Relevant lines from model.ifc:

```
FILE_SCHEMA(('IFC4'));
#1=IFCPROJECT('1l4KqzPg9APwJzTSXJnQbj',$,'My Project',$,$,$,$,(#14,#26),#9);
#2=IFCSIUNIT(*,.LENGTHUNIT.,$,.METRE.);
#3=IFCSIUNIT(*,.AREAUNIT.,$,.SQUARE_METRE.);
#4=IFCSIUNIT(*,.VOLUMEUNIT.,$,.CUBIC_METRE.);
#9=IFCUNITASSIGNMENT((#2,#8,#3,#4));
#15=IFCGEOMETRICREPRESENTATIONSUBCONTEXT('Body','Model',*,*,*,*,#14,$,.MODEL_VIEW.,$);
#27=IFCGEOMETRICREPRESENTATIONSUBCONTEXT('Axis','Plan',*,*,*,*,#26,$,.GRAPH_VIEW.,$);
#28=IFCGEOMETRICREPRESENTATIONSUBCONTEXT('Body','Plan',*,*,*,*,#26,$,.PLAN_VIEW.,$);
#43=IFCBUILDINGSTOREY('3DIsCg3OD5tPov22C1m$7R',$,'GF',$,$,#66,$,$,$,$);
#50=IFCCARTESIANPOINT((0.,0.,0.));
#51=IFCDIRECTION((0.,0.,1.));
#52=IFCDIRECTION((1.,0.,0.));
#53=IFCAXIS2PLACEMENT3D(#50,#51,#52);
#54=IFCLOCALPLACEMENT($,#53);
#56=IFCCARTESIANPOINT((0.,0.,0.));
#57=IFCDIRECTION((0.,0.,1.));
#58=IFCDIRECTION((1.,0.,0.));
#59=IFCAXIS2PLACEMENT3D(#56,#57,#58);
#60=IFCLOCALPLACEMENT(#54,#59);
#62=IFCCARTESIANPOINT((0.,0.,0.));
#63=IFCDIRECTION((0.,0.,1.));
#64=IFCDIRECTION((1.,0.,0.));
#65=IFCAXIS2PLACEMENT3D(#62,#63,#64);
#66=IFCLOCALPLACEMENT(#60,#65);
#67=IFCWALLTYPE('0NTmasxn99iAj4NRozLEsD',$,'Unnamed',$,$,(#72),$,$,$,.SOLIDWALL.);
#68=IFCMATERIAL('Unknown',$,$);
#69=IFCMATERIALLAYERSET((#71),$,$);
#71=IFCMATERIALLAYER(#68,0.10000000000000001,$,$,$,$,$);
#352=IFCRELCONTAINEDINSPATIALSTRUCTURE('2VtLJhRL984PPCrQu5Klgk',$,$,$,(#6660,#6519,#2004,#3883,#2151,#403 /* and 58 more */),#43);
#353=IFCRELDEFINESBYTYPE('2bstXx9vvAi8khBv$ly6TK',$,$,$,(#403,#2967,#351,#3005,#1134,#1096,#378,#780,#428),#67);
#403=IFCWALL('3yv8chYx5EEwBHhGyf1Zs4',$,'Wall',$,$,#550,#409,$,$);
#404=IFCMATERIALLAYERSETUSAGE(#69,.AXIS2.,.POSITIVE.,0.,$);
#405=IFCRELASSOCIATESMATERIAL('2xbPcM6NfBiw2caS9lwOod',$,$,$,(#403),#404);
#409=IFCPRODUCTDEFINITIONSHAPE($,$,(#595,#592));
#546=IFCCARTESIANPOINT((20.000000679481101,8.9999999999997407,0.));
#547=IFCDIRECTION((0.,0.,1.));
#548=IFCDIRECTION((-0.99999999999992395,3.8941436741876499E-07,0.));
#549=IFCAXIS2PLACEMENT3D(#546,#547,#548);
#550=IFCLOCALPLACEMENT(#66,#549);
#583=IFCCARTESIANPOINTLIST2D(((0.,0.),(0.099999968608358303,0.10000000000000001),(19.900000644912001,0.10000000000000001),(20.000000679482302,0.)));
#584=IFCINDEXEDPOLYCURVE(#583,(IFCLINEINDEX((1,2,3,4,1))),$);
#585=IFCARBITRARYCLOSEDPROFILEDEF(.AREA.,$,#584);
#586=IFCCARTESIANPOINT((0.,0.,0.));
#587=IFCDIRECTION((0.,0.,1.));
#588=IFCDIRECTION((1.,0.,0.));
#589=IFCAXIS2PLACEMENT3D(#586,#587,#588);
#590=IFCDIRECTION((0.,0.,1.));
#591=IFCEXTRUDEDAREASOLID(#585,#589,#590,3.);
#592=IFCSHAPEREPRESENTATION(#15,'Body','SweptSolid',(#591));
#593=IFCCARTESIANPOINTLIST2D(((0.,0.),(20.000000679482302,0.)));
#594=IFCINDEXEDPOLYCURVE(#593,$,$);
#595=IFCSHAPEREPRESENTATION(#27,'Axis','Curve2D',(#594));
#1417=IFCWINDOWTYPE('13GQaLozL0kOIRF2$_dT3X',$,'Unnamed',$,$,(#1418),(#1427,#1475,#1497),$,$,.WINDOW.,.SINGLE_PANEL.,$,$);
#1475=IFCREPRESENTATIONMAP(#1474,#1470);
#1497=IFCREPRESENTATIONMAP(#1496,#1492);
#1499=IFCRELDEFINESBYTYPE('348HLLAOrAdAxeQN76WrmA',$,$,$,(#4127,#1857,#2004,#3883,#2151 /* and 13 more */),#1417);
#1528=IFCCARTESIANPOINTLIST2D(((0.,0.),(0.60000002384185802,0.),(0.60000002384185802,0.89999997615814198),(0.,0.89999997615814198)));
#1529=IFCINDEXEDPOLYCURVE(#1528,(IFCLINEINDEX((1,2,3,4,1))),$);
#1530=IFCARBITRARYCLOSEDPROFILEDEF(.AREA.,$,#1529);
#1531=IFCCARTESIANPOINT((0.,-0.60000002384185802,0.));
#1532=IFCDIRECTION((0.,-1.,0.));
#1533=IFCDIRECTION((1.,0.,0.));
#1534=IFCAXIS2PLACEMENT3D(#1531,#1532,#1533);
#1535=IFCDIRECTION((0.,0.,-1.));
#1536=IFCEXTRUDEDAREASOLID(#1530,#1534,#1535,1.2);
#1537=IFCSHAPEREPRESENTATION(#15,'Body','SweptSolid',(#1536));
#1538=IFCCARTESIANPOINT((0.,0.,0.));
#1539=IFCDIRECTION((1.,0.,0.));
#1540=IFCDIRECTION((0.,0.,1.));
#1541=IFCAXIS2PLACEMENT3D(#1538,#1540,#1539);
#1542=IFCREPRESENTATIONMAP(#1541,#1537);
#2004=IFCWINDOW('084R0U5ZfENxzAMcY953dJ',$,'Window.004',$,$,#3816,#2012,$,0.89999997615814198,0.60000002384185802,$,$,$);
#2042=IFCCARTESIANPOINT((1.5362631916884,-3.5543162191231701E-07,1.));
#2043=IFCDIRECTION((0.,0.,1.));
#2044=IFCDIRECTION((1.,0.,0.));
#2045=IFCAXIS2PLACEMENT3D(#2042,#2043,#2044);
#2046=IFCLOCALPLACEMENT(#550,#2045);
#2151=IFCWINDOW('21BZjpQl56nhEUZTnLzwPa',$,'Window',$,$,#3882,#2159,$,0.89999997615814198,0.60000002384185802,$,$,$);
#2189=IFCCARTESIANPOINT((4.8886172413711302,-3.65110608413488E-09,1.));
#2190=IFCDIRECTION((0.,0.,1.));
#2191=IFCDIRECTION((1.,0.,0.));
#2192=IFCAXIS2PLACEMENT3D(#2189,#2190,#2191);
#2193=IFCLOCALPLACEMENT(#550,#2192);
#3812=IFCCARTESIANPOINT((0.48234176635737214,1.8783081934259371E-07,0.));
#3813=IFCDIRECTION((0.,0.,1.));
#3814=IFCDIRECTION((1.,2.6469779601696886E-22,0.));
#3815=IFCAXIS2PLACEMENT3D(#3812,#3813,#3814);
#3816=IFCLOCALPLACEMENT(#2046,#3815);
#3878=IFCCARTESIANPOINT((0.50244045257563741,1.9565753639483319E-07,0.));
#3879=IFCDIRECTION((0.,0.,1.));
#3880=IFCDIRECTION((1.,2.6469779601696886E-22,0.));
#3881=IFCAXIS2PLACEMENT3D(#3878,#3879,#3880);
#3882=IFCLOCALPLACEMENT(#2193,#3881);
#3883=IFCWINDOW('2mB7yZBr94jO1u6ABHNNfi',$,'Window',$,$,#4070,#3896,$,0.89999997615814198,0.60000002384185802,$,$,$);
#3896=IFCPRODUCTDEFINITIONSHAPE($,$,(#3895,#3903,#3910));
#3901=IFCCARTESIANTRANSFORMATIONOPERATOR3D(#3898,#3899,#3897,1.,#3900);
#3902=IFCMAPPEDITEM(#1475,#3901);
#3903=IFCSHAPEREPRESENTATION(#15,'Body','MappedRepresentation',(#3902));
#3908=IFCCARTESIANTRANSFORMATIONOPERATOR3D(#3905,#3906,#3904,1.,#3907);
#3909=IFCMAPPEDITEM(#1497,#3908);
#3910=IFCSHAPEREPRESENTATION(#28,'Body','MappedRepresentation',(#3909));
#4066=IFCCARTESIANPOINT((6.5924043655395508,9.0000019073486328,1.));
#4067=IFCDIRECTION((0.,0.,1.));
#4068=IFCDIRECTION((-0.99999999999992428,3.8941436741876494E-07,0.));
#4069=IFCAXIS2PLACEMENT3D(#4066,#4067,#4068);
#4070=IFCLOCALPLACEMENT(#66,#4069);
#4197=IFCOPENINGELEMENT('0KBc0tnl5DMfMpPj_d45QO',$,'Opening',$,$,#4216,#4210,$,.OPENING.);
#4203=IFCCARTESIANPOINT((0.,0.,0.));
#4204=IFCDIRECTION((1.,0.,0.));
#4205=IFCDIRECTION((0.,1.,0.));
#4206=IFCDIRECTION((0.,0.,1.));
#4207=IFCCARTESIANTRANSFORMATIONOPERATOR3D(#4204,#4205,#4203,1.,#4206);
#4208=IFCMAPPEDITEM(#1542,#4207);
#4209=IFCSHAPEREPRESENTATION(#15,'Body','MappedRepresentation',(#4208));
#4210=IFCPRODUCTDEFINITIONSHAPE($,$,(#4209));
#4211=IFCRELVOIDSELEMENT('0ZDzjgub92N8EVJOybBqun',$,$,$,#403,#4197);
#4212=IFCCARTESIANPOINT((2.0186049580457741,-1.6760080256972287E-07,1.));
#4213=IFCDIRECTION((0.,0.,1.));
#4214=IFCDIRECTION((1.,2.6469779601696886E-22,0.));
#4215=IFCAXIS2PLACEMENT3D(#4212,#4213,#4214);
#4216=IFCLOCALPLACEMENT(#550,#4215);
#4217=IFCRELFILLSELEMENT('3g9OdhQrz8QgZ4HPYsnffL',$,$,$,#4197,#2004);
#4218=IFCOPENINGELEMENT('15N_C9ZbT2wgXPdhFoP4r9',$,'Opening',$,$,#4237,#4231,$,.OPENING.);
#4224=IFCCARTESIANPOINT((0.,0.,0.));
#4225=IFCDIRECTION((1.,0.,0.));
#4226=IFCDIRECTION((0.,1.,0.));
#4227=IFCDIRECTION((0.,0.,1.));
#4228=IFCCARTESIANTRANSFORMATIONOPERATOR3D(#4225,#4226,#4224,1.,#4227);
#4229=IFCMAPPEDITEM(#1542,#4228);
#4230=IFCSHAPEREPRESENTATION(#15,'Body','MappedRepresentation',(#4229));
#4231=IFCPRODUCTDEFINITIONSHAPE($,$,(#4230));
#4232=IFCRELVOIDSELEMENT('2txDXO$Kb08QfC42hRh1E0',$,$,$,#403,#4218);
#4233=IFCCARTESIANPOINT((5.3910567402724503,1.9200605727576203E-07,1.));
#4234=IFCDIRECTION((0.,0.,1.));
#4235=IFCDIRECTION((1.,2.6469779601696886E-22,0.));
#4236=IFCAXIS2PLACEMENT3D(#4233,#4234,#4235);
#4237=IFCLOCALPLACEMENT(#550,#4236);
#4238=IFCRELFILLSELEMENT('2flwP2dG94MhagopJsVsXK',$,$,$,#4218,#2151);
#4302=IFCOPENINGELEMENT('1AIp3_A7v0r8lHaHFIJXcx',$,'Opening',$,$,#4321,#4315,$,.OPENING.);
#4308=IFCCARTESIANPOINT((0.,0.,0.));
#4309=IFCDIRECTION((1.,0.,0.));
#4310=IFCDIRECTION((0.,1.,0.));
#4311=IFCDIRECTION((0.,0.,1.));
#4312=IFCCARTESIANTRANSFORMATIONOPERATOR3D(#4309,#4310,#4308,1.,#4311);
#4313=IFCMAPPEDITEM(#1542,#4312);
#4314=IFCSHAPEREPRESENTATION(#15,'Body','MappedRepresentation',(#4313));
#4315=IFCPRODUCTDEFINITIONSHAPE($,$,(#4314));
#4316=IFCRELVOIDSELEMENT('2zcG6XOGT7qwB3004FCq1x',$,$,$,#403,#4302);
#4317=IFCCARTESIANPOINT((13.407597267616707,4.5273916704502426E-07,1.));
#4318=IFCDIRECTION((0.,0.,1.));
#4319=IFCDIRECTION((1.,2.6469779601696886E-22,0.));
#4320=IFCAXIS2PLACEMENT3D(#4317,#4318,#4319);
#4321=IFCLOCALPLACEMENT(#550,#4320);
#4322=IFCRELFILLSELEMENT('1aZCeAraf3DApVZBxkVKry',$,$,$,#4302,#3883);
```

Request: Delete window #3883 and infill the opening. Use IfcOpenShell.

```python
import ifcopenshell
import ifcopenshell.api.feature
import ifcopenshell.api.root
import ifcopenshell.geom
import ifcopenshell.util.shape

model = ifcopenshell.open("model.ifc")
settings = ifcopenshell.geom.settings()


def volume(element):
    """Net volume in cubic metres, openings subtracted."""
    shape = ifcopenshell.geom.create_shape(settings, element)
    return ifcopenshell.util.shape.get_volume(shape.geometry)


window = model.by_id(3883)
opening = window.FillsVoids[0].RelatingOpeningElement
wall = opening.VoidsElements[0].RelatingBuildingElement
before = volume(wall)

ifcopenshell.api.root.remove_product(model, product=window)
ifcopenshell.api.feature.remove_feature(model, feature=opening)

after = volume(wall)

print(f"wall volume {before:.3f} -> {after:.3f} m3")

model.write("model_v2.ifc")
```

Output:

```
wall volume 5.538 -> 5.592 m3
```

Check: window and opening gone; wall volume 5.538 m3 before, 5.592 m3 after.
